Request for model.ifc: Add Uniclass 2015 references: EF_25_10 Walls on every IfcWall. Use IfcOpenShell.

First a look at what the model holds.

```python
import ifcopenshell

model = ifcopenshell.open("model.ifc")
print(model.schema)
print("classifications:", [c.Name for c in model.by_type("IfcClassification")])
for ifc_class in ("IfcDoor", "IfcRoof", "IfcStair", "IfcWall", "IfcWindow"):
    print(ifc_class, len(model.by_type(ifc_class)))
```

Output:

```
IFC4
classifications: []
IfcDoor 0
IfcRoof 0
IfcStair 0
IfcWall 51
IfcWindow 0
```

```python
import ifcopenshell
import ifcopenshell.api.classification

model = ifcopenshell.open("model.ifc")

system = ifcopenshell.api.classification.add_classification(model, classification="Uniclass 2015")

codes = {
    "IfcWall": ("EF_25_10", "Walls"),
}
for ifc_class, (code, name) in codes.items():
    products = model.by_type(ifc_class)
    ifcopenshell.api.classification.add_reference(
        model, products=products, classification=system, identification=code, name=name
    )
    print(code, len(products))

model.write("model_v2.ifc")
```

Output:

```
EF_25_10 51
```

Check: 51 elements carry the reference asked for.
